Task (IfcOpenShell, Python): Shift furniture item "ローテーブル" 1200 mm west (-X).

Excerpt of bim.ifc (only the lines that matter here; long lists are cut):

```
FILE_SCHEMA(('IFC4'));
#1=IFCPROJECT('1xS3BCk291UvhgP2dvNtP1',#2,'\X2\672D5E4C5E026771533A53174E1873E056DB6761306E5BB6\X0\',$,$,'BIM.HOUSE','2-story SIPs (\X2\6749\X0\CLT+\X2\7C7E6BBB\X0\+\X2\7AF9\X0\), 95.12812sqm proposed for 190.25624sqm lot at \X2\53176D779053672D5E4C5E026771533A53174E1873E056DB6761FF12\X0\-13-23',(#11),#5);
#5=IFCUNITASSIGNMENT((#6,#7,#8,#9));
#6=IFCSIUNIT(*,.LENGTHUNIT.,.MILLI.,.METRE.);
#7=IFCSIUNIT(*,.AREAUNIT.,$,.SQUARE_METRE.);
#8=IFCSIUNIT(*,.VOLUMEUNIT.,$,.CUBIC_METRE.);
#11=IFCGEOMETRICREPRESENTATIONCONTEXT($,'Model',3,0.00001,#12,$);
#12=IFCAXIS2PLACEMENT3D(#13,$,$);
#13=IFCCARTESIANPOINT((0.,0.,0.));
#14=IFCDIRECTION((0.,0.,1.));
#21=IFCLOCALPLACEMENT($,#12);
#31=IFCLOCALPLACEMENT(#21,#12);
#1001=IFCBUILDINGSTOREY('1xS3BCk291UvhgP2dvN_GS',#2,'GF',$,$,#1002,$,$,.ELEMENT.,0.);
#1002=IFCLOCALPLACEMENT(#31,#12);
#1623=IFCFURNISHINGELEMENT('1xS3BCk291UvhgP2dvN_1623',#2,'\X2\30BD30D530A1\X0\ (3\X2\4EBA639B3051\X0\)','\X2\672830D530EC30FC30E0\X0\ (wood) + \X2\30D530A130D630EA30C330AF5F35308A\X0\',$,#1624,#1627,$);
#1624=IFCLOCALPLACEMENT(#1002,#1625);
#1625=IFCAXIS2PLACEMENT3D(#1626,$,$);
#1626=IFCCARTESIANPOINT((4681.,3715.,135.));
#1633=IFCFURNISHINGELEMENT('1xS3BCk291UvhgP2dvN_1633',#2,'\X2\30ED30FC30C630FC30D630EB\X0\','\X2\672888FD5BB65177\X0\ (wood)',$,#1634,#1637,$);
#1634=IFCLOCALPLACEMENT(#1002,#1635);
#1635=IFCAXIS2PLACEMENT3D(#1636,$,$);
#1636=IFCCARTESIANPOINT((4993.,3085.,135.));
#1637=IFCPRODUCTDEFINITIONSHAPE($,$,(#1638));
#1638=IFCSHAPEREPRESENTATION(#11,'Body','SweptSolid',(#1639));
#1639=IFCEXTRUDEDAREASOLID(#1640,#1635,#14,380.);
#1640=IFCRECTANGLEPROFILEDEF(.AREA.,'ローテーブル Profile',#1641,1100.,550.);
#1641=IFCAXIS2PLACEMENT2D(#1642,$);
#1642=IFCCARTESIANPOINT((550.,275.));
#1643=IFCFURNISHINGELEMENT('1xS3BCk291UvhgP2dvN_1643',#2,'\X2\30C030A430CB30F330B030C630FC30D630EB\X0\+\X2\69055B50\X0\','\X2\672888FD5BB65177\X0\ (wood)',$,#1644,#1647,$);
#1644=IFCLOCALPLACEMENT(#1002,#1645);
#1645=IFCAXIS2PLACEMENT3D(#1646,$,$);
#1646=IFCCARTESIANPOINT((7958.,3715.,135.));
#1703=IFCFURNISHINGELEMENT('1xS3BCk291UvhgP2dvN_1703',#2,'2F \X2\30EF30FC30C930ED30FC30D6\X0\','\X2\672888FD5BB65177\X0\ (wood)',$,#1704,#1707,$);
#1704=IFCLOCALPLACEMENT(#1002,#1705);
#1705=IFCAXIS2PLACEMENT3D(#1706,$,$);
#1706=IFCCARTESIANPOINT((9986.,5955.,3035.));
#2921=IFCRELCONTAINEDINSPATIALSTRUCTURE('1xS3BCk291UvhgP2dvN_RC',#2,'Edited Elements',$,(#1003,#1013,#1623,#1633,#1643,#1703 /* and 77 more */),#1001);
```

```python
import ifcopenshell
import ifcopenshell.api.geometry
import ifcopenshell.util.placement
import ifcopenshell.util.unit

model = ifcopenshell.open("bim.ifc")
unit_scale = ifcopenshell.util.unit.calculate_unit_scale(model)

item = model.by_guid("1xS3BCk291UvhgP2dvN_1633")
matrix = ifcopenshell.util.placement.get_local_placement(item.ObjectPlacement)
matrix[0, 3] -= 1.2 / unit_scale
ifcopenshell.api.geometry.edit_object_placement(model, product=item, matrix=matrix, is_si=False)

print(ifcopenshell.util.placement.get_local_placement(item.ObjectPlacement).round(3) + 0.0)

model.write("bim_edited.ifc")
```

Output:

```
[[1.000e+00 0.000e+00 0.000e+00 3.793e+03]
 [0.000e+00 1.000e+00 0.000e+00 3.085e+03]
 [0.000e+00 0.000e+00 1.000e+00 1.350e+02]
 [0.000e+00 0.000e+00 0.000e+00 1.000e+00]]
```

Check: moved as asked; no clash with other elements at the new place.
